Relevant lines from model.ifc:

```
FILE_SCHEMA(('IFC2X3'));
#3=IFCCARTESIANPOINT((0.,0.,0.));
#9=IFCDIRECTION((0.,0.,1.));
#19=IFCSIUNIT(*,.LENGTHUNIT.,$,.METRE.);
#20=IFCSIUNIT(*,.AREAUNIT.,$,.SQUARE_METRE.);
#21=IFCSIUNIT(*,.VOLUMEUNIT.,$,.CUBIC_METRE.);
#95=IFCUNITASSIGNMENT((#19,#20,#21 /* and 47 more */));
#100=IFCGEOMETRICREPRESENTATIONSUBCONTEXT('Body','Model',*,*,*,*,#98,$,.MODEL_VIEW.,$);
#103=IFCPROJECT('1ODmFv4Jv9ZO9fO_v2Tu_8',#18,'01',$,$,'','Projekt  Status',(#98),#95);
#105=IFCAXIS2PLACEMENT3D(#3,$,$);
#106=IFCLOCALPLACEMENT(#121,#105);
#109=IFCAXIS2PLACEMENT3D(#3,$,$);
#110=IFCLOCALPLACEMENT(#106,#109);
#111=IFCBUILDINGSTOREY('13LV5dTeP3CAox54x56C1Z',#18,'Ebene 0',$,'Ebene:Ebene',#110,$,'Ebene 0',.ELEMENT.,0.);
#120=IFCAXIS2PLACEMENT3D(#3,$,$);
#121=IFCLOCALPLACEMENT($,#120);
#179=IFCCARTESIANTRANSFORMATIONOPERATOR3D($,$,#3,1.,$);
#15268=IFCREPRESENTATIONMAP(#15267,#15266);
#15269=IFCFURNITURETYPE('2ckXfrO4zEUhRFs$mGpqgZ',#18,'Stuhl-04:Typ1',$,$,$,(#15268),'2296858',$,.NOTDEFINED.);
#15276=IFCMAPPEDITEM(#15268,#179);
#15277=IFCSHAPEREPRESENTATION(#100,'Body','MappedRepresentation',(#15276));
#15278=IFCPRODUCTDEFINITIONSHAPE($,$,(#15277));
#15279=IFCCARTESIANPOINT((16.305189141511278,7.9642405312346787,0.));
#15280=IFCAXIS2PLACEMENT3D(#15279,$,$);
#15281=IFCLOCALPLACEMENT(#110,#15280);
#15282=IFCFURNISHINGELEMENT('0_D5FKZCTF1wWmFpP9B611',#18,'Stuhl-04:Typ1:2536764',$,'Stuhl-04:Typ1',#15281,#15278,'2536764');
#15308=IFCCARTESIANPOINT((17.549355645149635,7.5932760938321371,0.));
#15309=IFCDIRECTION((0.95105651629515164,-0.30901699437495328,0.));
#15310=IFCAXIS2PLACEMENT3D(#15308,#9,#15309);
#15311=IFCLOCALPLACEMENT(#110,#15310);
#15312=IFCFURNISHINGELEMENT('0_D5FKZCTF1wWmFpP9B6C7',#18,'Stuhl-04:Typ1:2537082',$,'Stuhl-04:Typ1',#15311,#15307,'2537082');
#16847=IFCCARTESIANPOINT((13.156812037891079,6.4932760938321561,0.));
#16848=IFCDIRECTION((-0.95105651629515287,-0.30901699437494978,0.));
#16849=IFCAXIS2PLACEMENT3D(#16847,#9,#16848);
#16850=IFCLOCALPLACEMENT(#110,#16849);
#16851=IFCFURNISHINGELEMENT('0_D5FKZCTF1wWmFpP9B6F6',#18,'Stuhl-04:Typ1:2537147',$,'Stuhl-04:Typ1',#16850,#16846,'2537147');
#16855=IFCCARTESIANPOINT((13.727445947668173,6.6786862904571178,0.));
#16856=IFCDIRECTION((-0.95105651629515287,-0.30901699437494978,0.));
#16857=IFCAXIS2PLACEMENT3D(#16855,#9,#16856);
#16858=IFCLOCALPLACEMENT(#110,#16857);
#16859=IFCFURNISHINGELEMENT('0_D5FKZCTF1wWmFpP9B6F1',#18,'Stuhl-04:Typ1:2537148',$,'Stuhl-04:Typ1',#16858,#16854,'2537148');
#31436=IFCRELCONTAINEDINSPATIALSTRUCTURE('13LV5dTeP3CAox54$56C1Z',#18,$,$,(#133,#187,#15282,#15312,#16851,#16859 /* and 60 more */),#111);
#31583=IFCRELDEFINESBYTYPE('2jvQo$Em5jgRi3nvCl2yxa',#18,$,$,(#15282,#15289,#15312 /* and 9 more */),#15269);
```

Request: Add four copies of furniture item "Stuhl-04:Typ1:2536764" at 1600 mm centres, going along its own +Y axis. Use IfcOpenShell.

```python
import ifcopenshell
import ifcopenshell.api.geometry
import ifcopenshell.api.root
import ifcopenshell.util.element
import ifcopenshell.util.placement
import ifcopenshell.util.unit

model = ifcopenshell.open("model.ifc")
unit_scale = ifcopenshell.util.unit.calculate_unit_scale(model)

source = model.by_guid("0_D5FKZCTF1wWmFpP9B611")
base = ifcopenshell.util.placement.get_local_placement(source.ObjectPlacement)
step = base[:3, 1] * 1.6 / unit_scale

for i in range(1, 5):
    copy = ifcopenshell.api.root.copy_class(model, product=source)
    copy.Representation = ifcopenshell.util.element.copy_deep(
        model, source.Representation, exclude=["IfcGeometricRepresentationContext", "IfcRepresentationMap"]
    )
    copy.Name = "Stuhl-04:Typ1"
    copy.Tag = None
    matrix = base.copy()
    matrix[:3, 3] += i * step
    print("added at", matrix[:3, 3].round(3) + 0.0)
    ifcopenshell.api.geometry.edit_object_placement(model, product=copy, matrix=matrix, is_si=False)

model.write("model-out.ifc")
```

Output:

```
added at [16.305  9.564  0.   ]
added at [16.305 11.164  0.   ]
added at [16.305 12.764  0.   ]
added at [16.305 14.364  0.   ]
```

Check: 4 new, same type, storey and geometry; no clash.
